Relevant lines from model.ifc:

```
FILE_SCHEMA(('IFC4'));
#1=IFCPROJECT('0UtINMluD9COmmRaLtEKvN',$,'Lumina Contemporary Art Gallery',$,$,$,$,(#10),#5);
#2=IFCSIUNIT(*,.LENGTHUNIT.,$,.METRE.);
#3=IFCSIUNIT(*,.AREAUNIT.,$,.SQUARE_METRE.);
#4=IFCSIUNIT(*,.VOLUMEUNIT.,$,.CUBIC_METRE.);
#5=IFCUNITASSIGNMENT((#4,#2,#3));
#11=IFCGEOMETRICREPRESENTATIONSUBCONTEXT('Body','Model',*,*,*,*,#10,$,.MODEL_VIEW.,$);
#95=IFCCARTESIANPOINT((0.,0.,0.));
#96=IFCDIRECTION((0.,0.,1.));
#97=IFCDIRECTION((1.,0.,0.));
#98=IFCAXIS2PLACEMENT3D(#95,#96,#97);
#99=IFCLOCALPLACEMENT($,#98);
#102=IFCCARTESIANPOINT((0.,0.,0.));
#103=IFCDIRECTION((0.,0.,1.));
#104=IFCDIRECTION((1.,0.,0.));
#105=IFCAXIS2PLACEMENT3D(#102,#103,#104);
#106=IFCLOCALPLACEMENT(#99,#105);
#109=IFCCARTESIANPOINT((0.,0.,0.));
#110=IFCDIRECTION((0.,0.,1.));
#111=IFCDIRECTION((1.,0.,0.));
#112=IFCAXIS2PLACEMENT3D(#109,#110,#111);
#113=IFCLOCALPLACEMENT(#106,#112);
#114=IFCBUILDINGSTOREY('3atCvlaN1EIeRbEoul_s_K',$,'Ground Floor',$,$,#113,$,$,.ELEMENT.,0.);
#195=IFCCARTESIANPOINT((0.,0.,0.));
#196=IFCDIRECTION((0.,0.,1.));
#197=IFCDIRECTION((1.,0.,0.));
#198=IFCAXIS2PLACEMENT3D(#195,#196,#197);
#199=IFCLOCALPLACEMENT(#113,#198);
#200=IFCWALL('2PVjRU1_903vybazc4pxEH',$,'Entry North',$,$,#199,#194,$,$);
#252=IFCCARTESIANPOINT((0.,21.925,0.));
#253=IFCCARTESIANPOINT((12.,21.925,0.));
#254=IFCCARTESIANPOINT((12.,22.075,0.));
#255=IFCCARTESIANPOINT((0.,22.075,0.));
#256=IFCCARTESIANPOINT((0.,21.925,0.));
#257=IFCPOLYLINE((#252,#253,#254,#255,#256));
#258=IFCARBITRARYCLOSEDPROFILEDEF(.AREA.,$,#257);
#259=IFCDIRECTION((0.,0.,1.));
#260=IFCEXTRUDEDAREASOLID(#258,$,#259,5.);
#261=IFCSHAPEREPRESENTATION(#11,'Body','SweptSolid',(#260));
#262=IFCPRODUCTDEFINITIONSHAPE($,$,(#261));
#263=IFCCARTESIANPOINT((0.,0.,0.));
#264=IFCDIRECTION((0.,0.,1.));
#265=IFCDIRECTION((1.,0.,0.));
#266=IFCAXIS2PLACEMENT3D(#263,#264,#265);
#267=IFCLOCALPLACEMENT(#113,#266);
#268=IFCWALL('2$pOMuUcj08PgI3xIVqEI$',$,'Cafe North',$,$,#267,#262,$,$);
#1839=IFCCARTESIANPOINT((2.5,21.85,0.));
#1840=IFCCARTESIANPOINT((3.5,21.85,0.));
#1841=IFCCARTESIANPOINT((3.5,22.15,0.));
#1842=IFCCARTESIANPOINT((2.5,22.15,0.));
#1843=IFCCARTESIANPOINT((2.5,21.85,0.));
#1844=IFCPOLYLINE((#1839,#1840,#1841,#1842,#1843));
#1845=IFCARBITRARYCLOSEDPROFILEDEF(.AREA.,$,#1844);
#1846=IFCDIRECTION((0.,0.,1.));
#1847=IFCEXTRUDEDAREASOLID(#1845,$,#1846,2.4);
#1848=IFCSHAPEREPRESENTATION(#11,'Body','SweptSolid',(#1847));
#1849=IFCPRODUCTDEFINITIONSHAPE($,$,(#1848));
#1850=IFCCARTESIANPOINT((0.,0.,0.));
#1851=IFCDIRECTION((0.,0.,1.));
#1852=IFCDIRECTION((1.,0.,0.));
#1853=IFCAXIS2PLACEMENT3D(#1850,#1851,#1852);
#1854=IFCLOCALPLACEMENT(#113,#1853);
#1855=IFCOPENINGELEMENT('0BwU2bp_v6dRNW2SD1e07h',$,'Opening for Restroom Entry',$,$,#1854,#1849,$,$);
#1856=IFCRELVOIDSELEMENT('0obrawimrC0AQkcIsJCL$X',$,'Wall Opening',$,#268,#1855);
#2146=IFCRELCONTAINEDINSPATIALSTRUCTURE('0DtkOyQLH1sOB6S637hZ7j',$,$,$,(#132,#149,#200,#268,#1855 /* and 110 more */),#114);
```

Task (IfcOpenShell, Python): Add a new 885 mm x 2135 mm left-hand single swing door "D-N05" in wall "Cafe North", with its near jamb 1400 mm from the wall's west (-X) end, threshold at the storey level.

```python
import numpy as np
import ifcopenshell
import ifcopenshell.api.feature
import ifcopenshell.api.geometry
import ifcopenshell.api.root
import ifcopenshell.api.spatial
import ifcopenshell.geom
import ifcopenshell.util.element
import ifcopenshell.util.placement
import ifcopenshell.util.representation
import ifcopenshell.util.shape
import ifcopenshell.util.unit

model = ifcopenshell.open("model.ifc")
unit_scale = ifcopenshell.util.unit.calculate_unit_scale(model)
settings = ifcopenshell.geom.settings()


def volume(element):
    """Net volume in cubic metres, openings subtracted."""
    shape = ifcopenshell.geom.create_shape(settings, element)
    return ifcopenshell.util.shape.get_volume(shape.geometry)


wall = model.by_id(268)
storey = ifcopenshell.util.element.get_container(wall, ifc_class="IfcBuildingStorey")
context = ifcopenshell.util.representation.get_context(model, "Model", "Body", "MODEL_VIEW")
before = volume(wall)

width, height, from_end, sill = 0.885, 2.135, 1.4, 0.0  # metres

# The wall runs along its own X axis, and the end named is its -X end.
wall_shape = ifcopenshell.geom.create_shape(settings, wall)
x, y, z = ifcopenshell.util.shape.get_vertices(wall_shape.geometry).T
start = x.min() + from_end
face, thickness = float(y.min()), float(y.max() - y.min())
wall_matrix = ifcopenshell.util.placement.get_local_placement(wall.ObjectPlacement)
level = ifcopenshell.util.placement.get_local_placement(storey.ObjectPlacement)[2, 3]


def in_wall(x, y):
    """Placement at x, y metres in the wall's axes, at sill height."""
    matrix = wall_matrix.copy()
    matrix[:, 3] = wall_matrix @ np.array([x / unit_scale, y / unit_scale, 0.0, 1.0])
    matrix[2, 3] = level + sill / unit_scale
    return matrix


# Opening: a box that overshoots both wall faces by 50 mm.
opening = ifcopenshell.api.root.create_entity(model, ifc_class="IfcOpeningElement", predefined_type="OPENING")
box = ifcopenshell.api.geometry.add_wall_representation(
    model, context=context, length=width, height=height, thickness=thickness + 0.1
)
ifcopenshell.api.geometry.assign_representation(model, product=opening, representation=box)
ifcopenshell.api.geometry.edit_object_placement(model, product=opening, matrix=in_wall(start, face - 0.05), is_si=False)
ifcopenshell.api.feature.add_feature(model, feature=opening, element=wall)

door = ifcopenshell.api.root.create_entity(model, ifc_class="IfcDoor", name="D-N05", predefined_type="DOOR")
door.OverallWidth, door.OverallHeight = width / unit_scale, height / unit_scale
door.OperationType = "SINGLE_SWING_LEFT"
body = ifcopenshell.api.geometry.add_door_representation(
    model,
    context=context,
    overall_width=door.OverallWidth,
    overall_height=door.OverallHeight,
    operation_type="SINGLE_SWING_LEFT",
    lining_properties={"LiningDepth": thickness / unit_scale, "ThresholdDepth": thickness / unit_scale},
)
ifcopenshell.api.geometry.assign_representation(model, product=door, representation=body)
ifcopenshell.api.spatial.assign_container(model, products=[door], relating_structure=storey)
ifcopenshell.api.feature.add_filling(model, opening=opening, element=door)

# The lining spans the wall, so the door starts at the wall face.
ifcopenshell.api.geometry.edit_object_placement(model, product=door, matrix=in_wall(start, face), is_si=False)

after = volume(wall)

print(f"wall volume {before:.3f} -> {after:.3f} m3")

model.write("model_updated.ifc")
```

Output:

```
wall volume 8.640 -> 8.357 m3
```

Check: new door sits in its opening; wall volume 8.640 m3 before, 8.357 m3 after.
